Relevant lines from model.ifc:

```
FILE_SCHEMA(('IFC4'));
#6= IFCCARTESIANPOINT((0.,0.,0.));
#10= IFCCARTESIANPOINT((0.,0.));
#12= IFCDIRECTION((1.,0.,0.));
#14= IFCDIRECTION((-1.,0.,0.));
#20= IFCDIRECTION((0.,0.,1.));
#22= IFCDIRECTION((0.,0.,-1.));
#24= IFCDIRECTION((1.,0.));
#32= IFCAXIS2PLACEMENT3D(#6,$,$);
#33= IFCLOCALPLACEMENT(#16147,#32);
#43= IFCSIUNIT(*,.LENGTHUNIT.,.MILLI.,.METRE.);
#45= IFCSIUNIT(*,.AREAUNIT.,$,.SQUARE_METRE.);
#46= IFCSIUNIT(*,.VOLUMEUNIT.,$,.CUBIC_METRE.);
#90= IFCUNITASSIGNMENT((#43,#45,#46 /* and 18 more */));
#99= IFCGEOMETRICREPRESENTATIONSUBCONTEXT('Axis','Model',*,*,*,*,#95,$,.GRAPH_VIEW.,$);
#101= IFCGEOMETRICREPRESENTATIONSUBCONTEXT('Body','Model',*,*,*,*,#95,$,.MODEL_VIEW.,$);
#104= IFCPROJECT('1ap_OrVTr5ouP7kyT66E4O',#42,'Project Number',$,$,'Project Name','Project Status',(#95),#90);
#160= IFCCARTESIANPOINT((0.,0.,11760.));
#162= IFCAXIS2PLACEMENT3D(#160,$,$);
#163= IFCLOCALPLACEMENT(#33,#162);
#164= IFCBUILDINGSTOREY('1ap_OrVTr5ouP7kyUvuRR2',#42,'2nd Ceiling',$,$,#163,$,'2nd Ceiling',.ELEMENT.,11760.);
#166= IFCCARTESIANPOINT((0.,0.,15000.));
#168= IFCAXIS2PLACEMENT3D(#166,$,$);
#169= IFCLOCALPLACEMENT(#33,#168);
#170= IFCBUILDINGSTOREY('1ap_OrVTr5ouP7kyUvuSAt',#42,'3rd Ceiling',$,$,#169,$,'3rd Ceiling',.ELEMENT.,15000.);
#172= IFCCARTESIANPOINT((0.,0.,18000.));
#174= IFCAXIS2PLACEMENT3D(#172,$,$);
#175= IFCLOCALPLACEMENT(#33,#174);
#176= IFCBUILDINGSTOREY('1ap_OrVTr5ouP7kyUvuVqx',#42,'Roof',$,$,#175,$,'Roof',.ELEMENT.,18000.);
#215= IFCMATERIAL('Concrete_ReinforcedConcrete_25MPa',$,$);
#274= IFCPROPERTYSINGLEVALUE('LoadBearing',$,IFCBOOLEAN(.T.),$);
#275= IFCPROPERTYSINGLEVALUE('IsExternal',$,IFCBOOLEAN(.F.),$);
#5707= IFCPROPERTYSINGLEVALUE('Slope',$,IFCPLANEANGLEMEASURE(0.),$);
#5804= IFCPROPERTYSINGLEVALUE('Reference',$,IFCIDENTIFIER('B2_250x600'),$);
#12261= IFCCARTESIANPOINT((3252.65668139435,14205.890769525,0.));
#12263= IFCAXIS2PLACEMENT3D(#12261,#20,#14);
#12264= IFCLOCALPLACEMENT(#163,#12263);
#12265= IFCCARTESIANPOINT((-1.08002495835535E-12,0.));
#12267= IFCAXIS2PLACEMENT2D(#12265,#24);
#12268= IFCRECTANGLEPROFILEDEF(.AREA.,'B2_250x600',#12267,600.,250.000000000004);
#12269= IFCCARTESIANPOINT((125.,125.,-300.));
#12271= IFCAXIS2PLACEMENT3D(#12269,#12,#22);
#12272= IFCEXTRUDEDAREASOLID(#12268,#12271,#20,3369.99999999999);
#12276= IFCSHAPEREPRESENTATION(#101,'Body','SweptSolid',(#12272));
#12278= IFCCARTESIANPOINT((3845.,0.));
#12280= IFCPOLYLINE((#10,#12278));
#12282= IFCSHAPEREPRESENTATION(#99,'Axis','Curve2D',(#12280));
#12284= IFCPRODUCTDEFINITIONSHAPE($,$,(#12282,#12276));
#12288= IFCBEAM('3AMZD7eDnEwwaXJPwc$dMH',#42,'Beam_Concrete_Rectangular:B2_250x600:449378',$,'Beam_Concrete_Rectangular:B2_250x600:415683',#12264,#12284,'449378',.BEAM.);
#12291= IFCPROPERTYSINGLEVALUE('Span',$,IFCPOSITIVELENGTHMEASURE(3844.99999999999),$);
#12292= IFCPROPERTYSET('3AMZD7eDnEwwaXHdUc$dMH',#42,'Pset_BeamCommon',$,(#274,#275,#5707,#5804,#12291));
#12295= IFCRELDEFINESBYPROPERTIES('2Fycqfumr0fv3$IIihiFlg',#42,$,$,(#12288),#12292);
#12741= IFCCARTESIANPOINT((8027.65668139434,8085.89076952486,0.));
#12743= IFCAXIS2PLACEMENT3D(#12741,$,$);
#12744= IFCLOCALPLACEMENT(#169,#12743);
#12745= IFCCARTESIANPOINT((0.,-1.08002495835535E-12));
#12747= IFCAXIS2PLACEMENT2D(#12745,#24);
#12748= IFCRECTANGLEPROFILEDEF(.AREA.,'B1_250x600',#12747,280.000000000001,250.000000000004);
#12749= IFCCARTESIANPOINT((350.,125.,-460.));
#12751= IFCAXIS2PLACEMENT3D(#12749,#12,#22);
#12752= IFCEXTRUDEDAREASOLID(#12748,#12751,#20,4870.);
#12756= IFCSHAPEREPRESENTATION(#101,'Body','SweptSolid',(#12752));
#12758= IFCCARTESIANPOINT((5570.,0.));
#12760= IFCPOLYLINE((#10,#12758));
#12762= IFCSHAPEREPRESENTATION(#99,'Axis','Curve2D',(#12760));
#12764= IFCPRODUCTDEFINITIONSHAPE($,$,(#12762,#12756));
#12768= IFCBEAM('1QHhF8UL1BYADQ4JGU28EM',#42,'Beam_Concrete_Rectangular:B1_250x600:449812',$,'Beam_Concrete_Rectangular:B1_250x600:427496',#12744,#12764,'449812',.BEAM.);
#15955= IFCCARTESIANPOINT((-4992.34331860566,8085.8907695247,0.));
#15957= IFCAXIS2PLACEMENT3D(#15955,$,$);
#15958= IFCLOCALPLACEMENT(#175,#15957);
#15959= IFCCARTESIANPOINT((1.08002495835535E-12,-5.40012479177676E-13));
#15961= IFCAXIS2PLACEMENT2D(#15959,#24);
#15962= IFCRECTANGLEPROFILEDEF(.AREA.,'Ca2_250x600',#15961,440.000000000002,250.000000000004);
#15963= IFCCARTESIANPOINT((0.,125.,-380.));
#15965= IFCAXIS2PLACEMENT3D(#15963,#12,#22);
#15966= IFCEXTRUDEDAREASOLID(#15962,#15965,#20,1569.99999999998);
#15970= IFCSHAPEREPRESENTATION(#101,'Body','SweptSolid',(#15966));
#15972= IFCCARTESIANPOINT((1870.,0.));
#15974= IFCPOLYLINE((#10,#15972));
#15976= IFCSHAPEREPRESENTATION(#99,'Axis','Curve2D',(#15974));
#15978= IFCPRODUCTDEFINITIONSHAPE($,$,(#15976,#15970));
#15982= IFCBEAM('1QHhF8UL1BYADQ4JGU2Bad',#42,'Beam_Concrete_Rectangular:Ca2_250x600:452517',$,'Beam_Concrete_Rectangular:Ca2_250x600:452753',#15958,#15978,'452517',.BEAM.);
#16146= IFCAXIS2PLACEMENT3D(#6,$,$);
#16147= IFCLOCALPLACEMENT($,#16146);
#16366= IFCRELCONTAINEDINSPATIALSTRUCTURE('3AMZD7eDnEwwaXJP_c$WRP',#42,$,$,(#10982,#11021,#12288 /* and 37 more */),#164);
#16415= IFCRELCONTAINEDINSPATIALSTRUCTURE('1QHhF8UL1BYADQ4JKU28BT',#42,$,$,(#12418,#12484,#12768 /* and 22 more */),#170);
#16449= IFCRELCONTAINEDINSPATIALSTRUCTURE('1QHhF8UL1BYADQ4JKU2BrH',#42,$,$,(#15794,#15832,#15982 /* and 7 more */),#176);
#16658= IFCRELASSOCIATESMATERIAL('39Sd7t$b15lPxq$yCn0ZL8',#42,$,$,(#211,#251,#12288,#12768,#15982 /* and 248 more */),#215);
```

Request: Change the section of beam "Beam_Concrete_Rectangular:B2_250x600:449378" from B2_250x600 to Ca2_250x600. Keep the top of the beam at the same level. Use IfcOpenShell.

```python
import ifcopenshell
import ifcopenshell.api.pset
import ifcopenshell.util.element
import ifcopenshell.util.representation

model = ifcopenshell.open("model.ifc")

member = model.by_guid("3AMZD7eDnEwwaXJPwc$dMH")
source = next(p for p in model.by_type("IfcRectangleProfileDef") if p.ProfileName == "Ca2_250x600")

body = ifcopenshell.util.representation.get_representation(member, "Model", "Body")
solid = body.Items[0]
old_profile = solid.SweptArea

# Copy the section's sizes but keep this member's own profile position.
profile = ifcopenshell.util.element.copy(model, source)
# Profiles are centred, so shift by half the change in depth to hold the top.
shift = (old_profile.XDim - profile.XDim) / 2
x, y = old_profile.Position.Location.Coordinates
up = (-1.0, 0.0)  # upwards, in the solid's own plane
location = model.createIfcCartesianPoint((x + up[0] * shift, y + up[1] * shift))
profile.Position = model.createIfcAxis2Placement2D(location, old_profile.Position.RefDirection)
solid.SweptArea = profile
if not model.get_total_inverses(old_profile):
    ifcopenshell.util.element.remove_deep2(model, old_profile)
member.Name = member.Name.replace("B2_250x600", "Ca2_250x600")
member.ObjectType = member.ObjectType.replace("B2_250x600", "Ca2_250x600")
pset = model.by_id(ifcopenshell.util.element.get_pset(member, "Pset_BeamCommon", should_inherit=False)["id"])
ifcopenshell.api.pset.edit_pset(model, pset=pset, properties={"Reference": "Ca2_250x600"})

print(solid.SweptArea)

model.write("model_edited.ifc")
```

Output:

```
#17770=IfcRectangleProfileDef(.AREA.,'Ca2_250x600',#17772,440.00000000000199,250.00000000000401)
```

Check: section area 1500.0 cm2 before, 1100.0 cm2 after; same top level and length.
